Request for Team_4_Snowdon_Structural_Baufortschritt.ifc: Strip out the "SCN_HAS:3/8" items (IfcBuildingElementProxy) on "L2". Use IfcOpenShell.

First a look at what the model holds.

```python
import ifcopenshell
import ifcopenshell.util.element

model = ifcopenshell.open("Team_4_Snowdon_Structural_Baufortschritt.ifc")
print(model.schema)
storey = next(s for s in model.by_type("IfcBuildingStorey") if s.Name == "L2")
proxies = [e for e in ifcopenshell.util.element.get_decomposition(storey) if e.is_a("IfcBuildingElementProxy")]
seen = {}
for e in proxies:
    element_type = ifcopenshell.util.element.get_type(e)
    name = element_type.Name if element_type not in (None, e) else None
    seen[name] = seen.get(name, 0) + 1
for name, count in sorted(seen.items(), key=str):
    print(count, "x", name)
```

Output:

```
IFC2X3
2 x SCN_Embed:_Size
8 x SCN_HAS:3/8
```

```python
import ifcopenshell
import ifcopenshell.api.root
import ifcopenshell.util.element

model = ifcopenshell.open("Team_4_Snowdon_Structural_Baufortschritt.ifc")

storey = next(s for s in model.by_type("IfcBuildingStorey") if s.Name == "L2")
proxies = [e for e in ifcopenshell.util.element.get_decomposition(storey) if e.is_a("IfcBuildingElementProxy")]
targets = [e for e in proxies if (t := ifcopenshell.util.element.get_type(e)) not in (None, e) and t.Name == "SCN_HAS:3/8"]

for e in targets:
    ifcopenshell.api.root.remove_product(model, product=e)
print(len(targets), "removed")

model.write("Team_4_Snowdon_Structural_Baufortschritt_edited.ifc")
```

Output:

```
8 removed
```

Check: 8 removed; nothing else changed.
